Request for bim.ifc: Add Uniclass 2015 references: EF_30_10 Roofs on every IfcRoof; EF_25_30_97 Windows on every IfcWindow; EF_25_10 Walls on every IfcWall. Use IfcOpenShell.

First a look at what the model holds.

```python
import ifcopenshell

model = ifcopenshell.open("bim.ifc")
print(model.schema)
print("classifications:", [c.Name for c in model.by_type("IfcClassification")])
for ifc_class in ("IfcDoor", "IfcRoof", "IfcStair", "IfcWall", "IfcWindow"):
    print(ifc_class, len(model.by_type(ifc_class)))
```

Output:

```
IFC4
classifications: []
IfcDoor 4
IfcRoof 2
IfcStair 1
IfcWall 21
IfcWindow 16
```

```python
import ifcopenshell
import ifcopenshell.api.classification

model = ifcopenshell.open("bim.ifc")

system = ifcopenshell.api.classification.add_classification(model, classification="Uniclass 2015")

codes = {
    "IfcRoof": ("EF_30_10", "Roofs"),
    "IfcWindow": ("EF_25_30_97", "Windows"),
    "IfcWall": ("EF_25_10", "Walls"),
}
for ifc_class, (code, name) in codes.items():
    products = model.by_type(ifc_class)
    ifcopenshell.api.classification.add_reference(
        model, products=products, classification=system, identification=code, name=name
    )
    print(code, len(products))

model.write("bim_v2.ifc")
```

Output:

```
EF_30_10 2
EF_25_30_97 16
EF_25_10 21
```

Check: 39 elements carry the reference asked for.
